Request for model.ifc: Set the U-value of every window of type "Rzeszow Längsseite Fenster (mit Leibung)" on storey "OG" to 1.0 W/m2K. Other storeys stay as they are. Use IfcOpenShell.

First a look at what the model holds.

```python
import ifcopenshell
import ifcopenshell.util.element

model = ifcopenshell.open("model.ifc")
print(model.schema)
storey = next(s for s in model.by_type("IfcBuildingStorey") if s.Name == "OG")
windows = [e for e in ifcopenshell.util.element.get_decomposition(storey) if e.is_a("IfcWindow")]
seen = {}
for e in windows:
    element_type = ifcopenshell.util.element.get_type(e)
    key = (element_type.Name if element_type != e and element_type else None, ifcopenshell.util.element.get_pset(e, "Pset_WindowCommon", "ThermalTransmittance"))
    seen[key] = seen.get(key, 0) + 1
for (name, value), count in sorted(seen.items(), key=str):
    print(count, "x", name, "|", value)
```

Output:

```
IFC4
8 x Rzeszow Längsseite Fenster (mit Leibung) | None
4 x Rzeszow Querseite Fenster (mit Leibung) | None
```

```python
import ifcopenshell
import ifcopenshell.api.pset
import ifcopenshell.util.element

model = ifcopenshell.open("model.ifc")

storey = next(s for s in model.by_type("IfcBuildingStorey") if s.Name == "OG")
windows = [e for e in ifcopenshell.util.element.get_decomposition(storey) if e.is_a("IfcWindow")]

count = 0
for e in windows:
    element_type = ifcopenshell.util.element.get_type(e)
    if element_type in (None, e) or element_type.Name != "Rzeszow Längsseite Fenster (mit Leibung)":
        continue
    # add_pset returns the element's existing set when there is one.
    pset = ifcopenshell.api.pset.add_pset(model, product=e, name="Pset_WindowCommon")
    ifcopenshell.api.pset.edit_pset(model, pset=pset, properties={"ThermalTransmittance": 1.0})
    count += 1

print(count, "windows updated")

model.write("model_edited.ifc")
```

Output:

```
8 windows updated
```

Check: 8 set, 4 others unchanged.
